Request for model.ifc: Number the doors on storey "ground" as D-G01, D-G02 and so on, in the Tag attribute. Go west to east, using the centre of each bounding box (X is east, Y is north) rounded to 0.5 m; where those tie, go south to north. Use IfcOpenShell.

First a look at what the model holds.

```python
import ifcopenshell
import ifcopenshell.util.element
import ifcopenshell.util.placement

model = ifcopenshell.open("model.ifc")
print(model.schema)
storey = next(s for s in model.by_type("IfcBuildingStorey") if s.Name == "ground")
doors = [e for e in ifcopenshell.util.element.get_decomposition(storey) if e.is_a("IfcDoor")]
for e in sorted(doors, key=lambda e: e.id()):
    origin = ifcopenshell.util.placement.get_local_placement(e.ObjectPlacement)[:3, 3]
    print(e.id(), e.Tag, e.Name, origin.round(2) + 0.0, sep=" | ")
```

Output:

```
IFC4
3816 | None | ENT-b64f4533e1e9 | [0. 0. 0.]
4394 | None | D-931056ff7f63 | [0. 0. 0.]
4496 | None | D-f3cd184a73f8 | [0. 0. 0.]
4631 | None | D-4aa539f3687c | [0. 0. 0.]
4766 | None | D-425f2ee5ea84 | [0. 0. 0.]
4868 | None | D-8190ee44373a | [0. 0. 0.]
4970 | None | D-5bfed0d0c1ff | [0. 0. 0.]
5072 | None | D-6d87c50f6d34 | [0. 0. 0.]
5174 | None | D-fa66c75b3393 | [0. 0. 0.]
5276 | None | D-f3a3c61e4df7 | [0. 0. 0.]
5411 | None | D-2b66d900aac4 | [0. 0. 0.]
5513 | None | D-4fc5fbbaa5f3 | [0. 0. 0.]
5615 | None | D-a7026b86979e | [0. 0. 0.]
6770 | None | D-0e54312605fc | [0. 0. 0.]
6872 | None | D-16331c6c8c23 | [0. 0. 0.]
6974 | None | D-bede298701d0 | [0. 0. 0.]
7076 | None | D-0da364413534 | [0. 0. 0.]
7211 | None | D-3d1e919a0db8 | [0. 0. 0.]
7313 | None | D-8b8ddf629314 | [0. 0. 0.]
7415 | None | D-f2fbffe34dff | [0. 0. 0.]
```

```python
import ifcopenshell
import ifcopenshell.geom
import ifcopenshell.util.element
import ifcopenshell.util.shape

model = ifcopenshell.open("model.ifc")
settings = ifcopenshell.geom.settings()
settings.set("use-world-coords", True)


def centre(element):
    shape = ifcopenshell.geom.create_shape(settings, element)
    return ifcopenshell.util.shape.get_bbox_centroid(shape.geometry)


storey = next(s for s in model.by_type("IfcBuildingStorey") if s.Name == "ground")
doors = [e for e in ifcopenshell.util.element.get_decomposition(storey) if e.is_a("IfcDoor")]

# Insertion points can sit at a corner or the storey origin, so sort by the geometry (in metres).
centres = {e: centre(e) for e in doors}
doors.sort(key=lambda e: (round(centres[e][0] / 0.5), centres[e][1]))

for i, e in enumerate(doors, start=1):
    number = f"D-G{i:02d}"
    e.Tag = number
    print(e.id(), number)

model.write("model_updated.ifc")
```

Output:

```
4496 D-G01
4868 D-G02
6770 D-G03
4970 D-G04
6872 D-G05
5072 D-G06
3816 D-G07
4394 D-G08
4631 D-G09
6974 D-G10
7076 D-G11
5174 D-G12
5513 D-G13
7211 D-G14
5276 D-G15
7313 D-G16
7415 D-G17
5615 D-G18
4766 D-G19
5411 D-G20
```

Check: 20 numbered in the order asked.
